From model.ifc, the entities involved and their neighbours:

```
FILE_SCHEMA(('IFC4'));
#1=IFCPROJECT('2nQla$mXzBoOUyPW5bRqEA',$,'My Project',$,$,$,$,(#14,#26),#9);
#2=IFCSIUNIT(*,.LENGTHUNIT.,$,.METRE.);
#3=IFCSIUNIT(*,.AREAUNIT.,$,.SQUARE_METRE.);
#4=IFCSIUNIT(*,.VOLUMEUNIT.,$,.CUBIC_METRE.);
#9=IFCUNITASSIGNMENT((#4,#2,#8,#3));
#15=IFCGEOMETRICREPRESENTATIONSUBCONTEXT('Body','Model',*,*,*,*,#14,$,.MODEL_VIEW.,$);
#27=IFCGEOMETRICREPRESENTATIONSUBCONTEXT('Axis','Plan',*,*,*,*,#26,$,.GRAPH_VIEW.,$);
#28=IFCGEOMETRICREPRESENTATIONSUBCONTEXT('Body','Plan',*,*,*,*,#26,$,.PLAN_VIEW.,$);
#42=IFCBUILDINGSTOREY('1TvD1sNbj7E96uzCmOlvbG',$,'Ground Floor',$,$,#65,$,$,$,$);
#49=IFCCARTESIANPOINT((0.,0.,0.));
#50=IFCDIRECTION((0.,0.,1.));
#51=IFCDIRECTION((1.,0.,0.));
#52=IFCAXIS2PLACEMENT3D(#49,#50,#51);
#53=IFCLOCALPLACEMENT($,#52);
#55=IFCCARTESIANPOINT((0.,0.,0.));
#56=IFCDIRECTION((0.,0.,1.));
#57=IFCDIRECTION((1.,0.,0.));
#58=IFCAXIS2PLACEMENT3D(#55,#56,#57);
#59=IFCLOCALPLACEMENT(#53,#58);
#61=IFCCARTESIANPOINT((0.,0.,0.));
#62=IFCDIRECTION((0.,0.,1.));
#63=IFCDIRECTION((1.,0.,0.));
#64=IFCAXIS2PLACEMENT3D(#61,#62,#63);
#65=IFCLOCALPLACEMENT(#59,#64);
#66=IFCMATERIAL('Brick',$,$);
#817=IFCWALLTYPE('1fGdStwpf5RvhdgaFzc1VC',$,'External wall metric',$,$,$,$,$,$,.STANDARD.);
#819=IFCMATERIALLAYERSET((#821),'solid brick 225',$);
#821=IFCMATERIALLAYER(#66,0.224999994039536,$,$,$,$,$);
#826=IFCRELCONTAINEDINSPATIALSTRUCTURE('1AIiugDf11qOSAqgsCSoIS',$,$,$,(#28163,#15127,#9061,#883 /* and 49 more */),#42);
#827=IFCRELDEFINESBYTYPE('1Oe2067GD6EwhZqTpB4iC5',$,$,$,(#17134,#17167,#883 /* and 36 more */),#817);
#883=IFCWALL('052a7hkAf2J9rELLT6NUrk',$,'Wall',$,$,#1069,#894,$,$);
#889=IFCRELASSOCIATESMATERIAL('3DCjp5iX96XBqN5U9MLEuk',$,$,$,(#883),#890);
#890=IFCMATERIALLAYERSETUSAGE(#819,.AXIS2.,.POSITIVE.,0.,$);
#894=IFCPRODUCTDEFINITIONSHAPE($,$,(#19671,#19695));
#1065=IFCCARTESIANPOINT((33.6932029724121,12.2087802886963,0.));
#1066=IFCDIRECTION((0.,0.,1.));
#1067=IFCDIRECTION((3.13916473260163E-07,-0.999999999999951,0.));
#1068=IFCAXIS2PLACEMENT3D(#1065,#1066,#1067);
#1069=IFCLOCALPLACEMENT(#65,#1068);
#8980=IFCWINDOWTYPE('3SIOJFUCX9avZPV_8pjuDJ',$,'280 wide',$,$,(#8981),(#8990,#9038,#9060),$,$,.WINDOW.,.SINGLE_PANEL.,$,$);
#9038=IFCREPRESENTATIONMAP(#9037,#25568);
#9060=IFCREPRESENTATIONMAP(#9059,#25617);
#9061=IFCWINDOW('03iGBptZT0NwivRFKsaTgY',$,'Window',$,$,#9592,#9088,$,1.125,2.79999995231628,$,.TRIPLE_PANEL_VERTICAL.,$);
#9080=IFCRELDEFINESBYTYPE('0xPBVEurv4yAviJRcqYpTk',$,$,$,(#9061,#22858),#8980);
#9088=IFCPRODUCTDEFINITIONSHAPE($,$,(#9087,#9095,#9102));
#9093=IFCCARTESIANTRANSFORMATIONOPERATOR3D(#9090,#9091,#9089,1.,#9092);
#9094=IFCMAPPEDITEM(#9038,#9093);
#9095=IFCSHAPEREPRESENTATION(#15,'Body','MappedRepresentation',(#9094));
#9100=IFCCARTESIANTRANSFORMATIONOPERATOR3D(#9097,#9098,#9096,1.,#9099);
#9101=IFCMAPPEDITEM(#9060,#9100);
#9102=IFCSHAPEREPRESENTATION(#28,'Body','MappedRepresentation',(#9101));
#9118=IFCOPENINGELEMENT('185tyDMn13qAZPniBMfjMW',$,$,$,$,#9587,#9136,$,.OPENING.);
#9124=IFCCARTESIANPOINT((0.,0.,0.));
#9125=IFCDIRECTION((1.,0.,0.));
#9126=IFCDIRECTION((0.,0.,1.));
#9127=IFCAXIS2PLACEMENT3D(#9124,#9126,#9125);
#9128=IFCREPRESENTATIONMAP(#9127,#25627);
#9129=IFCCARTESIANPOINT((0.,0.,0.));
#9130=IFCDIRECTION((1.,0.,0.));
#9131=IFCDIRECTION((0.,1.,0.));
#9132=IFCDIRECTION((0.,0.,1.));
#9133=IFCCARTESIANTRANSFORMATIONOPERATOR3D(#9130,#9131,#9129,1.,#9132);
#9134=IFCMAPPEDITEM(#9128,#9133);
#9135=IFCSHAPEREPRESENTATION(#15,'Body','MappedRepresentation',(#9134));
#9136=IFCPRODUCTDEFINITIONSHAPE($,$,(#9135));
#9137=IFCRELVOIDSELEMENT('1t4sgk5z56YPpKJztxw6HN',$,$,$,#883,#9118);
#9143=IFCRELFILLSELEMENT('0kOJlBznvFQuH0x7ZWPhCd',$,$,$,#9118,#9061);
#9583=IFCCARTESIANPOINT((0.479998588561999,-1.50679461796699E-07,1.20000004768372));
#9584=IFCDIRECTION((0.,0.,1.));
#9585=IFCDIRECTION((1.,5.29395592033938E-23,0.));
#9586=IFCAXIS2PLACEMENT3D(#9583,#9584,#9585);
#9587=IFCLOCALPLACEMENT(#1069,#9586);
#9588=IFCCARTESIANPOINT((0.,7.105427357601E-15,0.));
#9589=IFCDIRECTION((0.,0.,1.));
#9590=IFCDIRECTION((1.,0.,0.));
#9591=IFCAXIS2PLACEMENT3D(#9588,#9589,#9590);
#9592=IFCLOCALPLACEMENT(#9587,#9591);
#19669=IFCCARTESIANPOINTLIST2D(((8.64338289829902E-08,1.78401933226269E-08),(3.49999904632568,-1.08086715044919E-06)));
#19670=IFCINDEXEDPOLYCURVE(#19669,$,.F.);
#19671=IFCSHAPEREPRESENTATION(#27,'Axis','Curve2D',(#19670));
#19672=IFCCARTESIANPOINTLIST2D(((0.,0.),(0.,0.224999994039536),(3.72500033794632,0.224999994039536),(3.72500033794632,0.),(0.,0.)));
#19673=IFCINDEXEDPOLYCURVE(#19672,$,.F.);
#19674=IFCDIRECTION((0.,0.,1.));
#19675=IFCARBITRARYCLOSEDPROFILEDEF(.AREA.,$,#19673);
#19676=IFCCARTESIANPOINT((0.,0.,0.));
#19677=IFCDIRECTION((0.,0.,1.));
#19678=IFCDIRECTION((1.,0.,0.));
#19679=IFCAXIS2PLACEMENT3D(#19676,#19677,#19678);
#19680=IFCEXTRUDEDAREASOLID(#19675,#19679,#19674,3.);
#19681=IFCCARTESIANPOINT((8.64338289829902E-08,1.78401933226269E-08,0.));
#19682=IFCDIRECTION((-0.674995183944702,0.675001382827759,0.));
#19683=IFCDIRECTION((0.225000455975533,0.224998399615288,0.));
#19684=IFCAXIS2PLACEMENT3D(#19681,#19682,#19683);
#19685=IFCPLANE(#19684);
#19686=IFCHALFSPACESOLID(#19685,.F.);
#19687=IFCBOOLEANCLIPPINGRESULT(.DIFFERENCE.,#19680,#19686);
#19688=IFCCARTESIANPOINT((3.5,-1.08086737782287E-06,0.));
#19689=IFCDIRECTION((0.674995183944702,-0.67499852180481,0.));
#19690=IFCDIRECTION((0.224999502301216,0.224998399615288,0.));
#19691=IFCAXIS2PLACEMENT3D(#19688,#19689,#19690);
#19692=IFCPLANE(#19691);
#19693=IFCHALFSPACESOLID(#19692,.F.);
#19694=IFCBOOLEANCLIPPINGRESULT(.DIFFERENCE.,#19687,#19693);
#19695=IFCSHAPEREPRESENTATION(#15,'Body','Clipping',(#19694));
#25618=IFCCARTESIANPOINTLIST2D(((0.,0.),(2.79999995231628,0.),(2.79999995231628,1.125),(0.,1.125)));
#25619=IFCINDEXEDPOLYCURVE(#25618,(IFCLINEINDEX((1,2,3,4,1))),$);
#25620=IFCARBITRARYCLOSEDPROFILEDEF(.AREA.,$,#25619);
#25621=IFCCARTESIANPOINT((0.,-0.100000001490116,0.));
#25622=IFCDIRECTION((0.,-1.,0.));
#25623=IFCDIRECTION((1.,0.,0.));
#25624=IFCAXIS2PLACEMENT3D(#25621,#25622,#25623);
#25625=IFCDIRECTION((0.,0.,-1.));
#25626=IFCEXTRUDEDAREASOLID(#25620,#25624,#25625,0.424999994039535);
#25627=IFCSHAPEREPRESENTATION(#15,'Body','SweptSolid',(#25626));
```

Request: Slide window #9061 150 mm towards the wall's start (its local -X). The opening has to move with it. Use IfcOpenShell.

```python
import ifcopenshell
import ifcopenshell.api.geometry
import ifcopenshell.util.placement
import ifcopenshell.util.unit

model = ifcopenshell.open("model.ifc")
unit_scale = ifcopenshell.util.unit.calculate_unit_scale(model)

window = model.by_id(9061)
opening = window.FillsVoids[0].RelatingOpeningElement
wall = opening.VoidsElements[0].RelatingBuildingElement

wall_matrix = ifcopenshell.util.placement.get_local_placement(wall.ObjectPlacement)
shift = wall_matrix[:3, 0] * -0.15 / unit_scale
before = ifcopenshell.util.placement.get_local_placement(window.ObjectPlacement)[:3, 3].copy()

# The window is placed relative to its opening, so it follows when the opening moves.
matrix = ifcopenshell.util.placement.get_local_placement(opening.ObjectPlacement)
matrix[:3, 3] += shift
ifcopenshell.api.geometry.edit_object_placement(
    model, product=opening, matrix=matrix, is_si=False, should_transform_children=True
)

after = ifcopenshell.util.placement.get_local_placement(window.ObjectPlacement)[:3, 3]
print("window moved by", (after - before).round(3) + 0.0)

model.write("model_rev.ifc")
```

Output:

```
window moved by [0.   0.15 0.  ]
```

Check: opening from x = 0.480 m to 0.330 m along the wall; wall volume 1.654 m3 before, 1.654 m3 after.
